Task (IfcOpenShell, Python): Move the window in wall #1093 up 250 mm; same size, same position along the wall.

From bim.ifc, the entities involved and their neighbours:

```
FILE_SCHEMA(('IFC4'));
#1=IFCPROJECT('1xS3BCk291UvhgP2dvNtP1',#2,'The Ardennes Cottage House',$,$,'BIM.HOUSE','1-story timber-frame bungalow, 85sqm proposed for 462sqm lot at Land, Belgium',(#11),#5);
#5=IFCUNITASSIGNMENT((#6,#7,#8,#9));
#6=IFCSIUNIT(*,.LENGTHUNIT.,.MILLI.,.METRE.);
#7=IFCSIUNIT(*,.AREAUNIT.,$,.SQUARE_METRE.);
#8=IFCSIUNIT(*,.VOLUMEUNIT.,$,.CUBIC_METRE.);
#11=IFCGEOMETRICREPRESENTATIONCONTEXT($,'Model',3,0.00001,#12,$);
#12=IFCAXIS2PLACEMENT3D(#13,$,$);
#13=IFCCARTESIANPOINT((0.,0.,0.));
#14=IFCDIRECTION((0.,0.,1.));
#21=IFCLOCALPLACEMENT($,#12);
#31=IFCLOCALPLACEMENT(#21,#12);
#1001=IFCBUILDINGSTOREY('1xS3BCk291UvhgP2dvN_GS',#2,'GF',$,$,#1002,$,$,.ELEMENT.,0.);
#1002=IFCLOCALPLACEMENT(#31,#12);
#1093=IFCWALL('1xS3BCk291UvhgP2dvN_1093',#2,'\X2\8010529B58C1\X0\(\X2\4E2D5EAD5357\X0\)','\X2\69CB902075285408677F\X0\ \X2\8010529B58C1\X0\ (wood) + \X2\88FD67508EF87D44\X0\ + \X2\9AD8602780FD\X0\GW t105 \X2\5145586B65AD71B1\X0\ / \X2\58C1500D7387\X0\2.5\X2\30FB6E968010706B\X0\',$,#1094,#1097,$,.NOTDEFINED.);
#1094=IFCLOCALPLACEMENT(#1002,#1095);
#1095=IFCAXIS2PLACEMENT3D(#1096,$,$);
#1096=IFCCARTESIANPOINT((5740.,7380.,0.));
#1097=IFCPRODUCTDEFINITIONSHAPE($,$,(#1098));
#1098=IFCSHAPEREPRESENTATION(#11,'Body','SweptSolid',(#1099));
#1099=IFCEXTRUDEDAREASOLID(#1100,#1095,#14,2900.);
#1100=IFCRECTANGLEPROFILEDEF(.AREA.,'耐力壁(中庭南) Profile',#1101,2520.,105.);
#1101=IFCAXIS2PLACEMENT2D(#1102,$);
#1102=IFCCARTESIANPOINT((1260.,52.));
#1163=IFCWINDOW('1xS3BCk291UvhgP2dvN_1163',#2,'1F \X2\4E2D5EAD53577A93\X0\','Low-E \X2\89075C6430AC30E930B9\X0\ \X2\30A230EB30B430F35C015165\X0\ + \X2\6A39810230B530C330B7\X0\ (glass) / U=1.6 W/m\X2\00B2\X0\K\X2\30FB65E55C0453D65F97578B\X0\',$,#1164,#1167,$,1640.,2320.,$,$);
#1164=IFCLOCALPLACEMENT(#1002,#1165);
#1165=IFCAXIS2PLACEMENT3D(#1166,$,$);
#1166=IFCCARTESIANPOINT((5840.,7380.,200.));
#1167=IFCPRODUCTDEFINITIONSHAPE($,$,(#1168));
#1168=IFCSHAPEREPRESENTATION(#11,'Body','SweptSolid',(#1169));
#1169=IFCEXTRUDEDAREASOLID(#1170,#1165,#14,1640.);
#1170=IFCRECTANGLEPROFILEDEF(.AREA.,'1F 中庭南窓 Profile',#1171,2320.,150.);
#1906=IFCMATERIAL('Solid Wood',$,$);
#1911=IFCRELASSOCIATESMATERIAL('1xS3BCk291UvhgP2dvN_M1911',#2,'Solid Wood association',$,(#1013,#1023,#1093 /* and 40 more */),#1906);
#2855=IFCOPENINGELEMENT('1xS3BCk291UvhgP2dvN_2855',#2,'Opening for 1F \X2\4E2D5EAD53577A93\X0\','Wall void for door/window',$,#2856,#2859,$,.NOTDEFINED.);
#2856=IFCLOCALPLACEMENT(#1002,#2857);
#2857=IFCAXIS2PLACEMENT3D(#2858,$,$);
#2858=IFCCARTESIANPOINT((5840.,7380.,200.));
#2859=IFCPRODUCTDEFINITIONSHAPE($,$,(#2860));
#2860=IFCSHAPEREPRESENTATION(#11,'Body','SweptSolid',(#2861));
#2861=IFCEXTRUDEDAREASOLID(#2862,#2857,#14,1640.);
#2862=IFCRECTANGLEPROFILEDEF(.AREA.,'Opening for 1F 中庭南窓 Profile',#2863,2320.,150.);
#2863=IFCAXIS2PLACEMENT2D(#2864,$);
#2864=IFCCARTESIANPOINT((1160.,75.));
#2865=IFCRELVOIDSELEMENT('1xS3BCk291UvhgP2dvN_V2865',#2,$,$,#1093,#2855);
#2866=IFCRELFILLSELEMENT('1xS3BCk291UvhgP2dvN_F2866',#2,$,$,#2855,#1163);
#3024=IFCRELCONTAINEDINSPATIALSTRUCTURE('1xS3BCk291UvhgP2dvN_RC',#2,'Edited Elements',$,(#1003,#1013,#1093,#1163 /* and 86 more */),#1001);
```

```python
import numpy as np
import ifcopenshell
import ifcopenshell.api.geometry
import ifcopenshell.util.placement
import ifcopenshell.util.unit

model = ifcopenshell.open("bim.ifc")
unit_scale = ifcopenshell.util.unit.calculate_unit_scale(model)

window = model.by_id(1163)
opening = window.FillsVoids[0].RelatingOpeningElement
dz = 0.25 / unit_scale

shift = np.array([0.0, 0.0, dz])
# The window is not placed relative to its opening, so move both.
for product in (opening, window):
    matrix = ifcopenshell.util.placement.get_local_placement(product.ObjectPlacement)
    matrix[:3, 3] += shift
    ifcopenshell.api.geometry.edit_object_placement(model, product=product, matrix=matrix, is_si=False)

print(f"moved by {dz * unit_scale:+.3f} m")

model.write("bim_updated.ifc")
```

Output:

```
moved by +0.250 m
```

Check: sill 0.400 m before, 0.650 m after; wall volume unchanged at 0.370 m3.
